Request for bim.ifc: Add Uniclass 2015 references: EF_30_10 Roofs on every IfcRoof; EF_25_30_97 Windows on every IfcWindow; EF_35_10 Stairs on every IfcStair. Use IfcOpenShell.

First a look at what the model holds.

```python
import ifcopenshell

model = ifcopenshell.open("bim.ifc")
print(model.schema)
print("classifications:", [c.Name for c in model.by_type("IfcClassification")])
for ifc_class in ("IfcDoor", "IfcRoof", "IfcStair", "IfcWall", "IfcWindow"):
    print(ifc_class, len(model.by_type(ifc_class)))
```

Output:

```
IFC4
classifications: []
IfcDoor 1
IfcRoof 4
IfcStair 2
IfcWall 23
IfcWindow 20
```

```python
import ifcopenshell
import ifcopenshell.api.classification

model = ifcopenshell.open("bim.ifc")

system = ifcopenshell.api.classification.add_classification(model, classification="Uniclass 2015")

codes = {
    "IfcRoof": ("EF_30_10", "Roofs"),
    "IfcWindow": ("EF_25_30_97", "Windows"),
    "IfcStair": ("EF_35_10", "Stairs"),
}
for ifc_class, (code, name) in codes.items():
    products = model.by_type(ifc_class)
    ifcopenshell.api.classification.add_reference(
        model, products=products, classification=system, identification=code, name=name
    )
    print(code, len(products))

model.write("bim-out.ifc")
```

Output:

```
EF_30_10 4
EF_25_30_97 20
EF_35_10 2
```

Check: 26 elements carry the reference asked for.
